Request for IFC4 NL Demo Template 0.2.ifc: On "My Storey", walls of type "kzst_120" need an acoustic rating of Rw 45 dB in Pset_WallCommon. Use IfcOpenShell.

First a look at what the model holds.

```python
import ifcopenshell
import ifcopenshell.util.element

model = ifcopenshell.open("IFC4 NL Demo Template 0.2.ifc")
print(model.schema)
storey = next(s for s in model.by_type("IfcBuildingStorey") if s.Name == "My Storey")
walls = [e for e in ifcopenshell.util.element.get_decomposition(storey) if e.is_a("IfcWall")]
seen = {}
for e in walls:
    element_type = ifcopenshell.util.element.get_type(e)
    key = (element_type.Name if element_type != e and element_type else None, ifcopenshell.util.element.get_pset(e, "Pset_WallCommon", "AcousticRating"))
    seen[key] = seen.get(key, 0) + 1
for (name, value), count in sorted(seen.items(), key=str):
    print(count, "x", name, "|", value)
```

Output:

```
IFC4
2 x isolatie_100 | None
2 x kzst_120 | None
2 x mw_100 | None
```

```python
import ifcopenshell
import ifcopenshell.api.pset
import ifcopenshell.util.element

model = ifcopenshell.open("IFC4 NL Demo Template 0.2.ifc")

storey = next(s for s in model.by_type("IfcBuildingStorey") if s.Name == "My Storey")
walls = [e for e in ifcopenshell.util.element.get_decomposition(storey) if e.is_a("IfcWall")]

count = 0
for e in walls:
    element_type = ifcopenshell.util.element.get_type(e)
    if element_type in (None, e) or element_type.Name != "kzst_120":
        continue
    # add_pset returns the element's existing set when there is one.
    pset = ifcopenshell.api.pset.add_pset(model, product=e, name="Pset_WallCommon")
    ifcopenshell.api.pset.edit_pset(model, pset=pset, properties={"AcousticRating": "Rw 45 dB"})
    count += 1

print(count, "walls updated")

model.write("IFC4 NL Demo Template 0.2-out.ifc")
```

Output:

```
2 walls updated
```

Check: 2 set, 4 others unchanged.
